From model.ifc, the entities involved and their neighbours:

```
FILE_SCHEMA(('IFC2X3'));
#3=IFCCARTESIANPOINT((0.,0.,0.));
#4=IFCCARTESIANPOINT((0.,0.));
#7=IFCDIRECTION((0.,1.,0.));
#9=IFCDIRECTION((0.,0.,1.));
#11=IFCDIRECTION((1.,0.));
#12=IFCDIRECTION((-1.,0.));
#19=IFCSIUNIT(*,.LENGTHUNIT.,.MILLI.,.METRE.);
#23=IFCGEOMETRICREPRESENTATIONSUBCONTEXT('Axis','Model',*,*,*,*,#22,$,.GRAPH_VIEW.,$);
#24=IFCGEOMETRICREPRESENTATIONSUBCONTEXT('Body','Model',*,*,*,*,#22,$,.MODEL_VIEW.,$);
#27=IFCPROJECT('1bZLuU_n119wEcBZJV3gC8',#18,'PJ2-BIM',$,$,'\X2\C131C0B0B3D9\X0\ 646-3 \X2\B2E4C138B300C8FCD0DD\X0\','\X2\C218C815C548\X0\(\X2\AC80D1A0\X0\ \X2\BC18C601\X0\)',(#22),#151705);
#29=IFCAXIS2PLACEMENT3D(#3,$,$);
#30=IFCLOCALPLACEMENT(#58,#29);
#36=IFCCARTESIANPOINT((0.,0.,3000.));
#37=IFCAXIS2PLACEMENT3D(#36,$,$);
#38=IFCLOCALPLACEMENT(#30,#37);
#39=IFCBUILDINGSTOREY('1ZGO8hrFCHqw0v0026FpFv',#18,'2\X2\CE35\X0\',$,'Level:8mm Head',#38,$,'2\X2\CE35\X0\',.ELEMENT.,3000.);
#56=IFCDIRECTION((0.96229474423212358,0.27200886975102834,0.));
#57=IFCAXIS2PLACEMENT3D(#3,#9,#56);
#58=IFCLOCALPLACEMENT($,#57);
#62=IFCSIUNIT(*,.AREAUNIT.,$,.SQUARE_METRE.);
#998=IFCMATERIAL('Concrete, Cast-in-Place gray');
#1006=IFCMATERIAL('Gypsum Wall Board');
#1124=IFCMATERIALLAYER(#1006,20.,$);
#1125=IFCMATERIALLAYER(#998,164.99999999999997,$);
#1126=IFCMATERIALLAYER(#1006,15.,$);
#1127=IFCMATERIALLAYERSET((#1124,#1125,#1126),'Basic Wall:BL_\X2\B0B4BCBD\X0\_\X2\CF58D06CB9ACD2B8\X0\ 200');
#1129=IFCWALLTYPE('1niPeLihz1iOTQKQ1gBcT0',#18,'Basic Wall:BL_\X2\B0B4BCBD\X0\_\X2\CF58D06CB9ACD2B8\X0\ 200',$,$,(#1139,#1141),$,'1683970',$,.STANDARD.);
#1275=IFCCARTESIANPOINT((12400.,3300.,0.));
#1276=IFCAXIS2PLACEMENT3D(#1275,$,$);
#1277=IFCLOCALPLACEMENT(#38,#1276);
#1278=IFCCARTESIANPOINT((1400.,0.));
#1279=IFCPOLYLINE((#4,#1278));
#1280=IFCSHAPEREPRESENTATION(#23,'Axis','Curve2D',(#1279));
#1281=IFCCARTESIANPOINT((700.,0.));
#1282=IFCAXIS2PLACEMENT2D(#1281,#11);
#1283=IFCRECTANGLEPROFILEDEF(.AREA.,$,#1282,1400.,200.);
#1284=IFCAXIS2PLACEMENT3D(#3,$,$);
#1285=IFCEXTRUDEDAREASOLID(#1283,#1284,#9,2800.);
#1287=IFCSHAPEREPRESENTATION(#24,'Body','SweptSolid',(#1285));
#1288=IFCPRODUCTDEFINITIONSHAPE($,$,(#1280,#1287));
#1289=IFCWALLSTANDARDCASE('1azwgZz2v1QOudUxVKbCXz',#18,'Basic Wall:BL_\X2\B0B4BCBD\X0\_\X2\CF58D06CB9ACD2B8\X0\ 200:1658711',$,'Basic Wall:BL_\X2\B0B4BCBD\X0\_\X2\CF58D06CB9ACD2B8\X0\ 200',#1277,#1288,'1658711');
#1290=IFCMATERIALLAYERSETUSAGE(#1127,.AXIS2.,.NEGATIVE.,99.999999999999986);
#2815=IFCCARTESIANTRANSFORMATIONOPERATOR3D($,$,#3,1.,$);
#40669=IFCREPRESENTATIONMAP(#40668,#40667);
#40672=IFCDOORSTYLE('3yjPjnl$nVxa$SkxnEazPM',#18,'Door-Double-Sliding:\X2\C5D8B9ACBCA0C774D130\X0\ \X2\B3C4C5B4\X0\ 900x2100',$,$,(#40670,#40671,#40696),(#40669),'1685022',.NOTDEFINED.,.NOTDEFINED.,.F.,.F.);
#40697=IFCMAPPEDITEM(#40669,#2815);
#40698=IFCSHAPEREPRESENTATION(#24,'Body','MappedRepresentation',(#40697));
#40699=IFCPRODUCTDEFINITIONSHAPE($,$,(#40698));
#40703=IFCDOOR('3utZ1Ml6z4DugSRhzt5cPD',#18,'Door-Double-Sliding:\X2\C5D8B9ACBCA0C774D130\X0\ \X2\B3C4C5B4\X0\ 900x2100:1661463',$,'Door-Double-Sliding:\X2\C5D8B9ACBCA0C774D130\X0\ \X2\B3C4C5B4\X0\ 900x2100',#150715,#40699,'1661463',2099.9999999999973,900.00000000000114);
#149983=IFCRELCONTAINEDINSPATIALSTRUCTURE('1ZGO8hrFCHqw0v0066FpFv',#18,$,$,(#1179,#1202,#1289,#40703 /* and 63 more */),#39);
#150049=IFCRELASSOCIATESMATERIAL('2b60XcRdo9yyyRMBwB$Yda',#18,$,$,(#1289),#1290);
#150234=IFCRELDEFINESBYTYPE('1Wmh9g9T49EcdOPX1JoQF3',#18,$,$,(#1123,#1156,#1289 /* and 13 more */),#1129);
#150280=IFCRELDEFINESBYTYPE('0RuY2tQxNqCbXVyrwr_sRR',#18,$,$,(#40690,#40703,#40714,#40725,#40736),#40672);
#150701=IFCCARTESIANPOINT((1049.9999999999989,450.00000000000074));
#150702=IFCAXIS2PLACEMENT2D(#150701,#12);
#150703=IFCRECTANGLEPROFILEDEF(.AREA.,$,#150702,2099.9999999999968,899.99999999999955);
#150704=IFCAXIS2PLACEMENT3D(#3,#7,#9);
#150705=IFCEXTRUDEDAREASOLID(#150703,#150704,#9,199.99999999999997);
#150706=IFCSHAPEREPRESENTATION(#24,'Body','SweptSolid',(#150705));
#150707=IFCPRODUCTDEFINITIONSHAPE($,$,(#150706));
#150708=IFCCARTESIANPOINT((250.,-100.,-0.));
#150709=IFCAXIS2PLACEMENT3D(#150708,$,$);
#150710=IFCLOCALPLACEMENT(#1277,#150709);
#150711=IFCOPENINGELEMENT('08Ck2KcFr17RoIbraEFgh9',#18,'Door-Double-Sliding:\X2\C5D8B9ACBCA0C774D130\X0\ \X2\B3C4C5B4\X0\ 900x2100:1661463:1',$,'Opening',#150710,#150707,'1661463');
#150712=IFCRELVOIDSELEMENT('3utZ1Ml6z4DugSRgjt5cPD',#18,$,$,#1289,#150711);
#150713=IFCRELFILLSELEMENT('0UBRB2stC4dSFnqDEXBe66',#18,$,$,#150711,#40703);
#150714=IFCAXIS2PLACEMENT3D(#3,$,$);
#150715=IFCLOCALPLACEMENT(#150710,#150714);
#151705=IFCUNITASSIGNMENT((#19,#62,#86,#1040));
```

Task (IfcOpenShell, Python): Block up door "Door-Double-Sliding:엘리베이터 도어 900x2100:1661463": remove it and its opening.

```python
import ifcopenshell
import ifcopenshell.api.feature
import ifcopenshell.api.root
import ifcopenshell.geom
import ifcopenshell.util.shape

model = ifcopenshell.open("model.ifc")
settings = ifcopenshell.geom.settings()


def volume(element):
    """Net volume in cubic metres, openings subtracted."""
    shape = ifcopenshell.geom.create_shape(settings, element)
    return ifcopenshell.util.shape.get_volume(shape.geometry)


door = model.by_id(40703)
opening = door.FillsVoids[0].RelatingOpeningElement
wall = opening.VoidsElements[0].RelatingBuildingElement
before = volume(wall)

ifcopenshell.api.root.remove_product(model, product=door)
ifcopenshell.api.feature.remove_feature(model, feature=opening)

after = volume(wall)

print(f"wall volume {before:.3f} -> {after:.3f} m3")

model.write("model_rev.ifc")
```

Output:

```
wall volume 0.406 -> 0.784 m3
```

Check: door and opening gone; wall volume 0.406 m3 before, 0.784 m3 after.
